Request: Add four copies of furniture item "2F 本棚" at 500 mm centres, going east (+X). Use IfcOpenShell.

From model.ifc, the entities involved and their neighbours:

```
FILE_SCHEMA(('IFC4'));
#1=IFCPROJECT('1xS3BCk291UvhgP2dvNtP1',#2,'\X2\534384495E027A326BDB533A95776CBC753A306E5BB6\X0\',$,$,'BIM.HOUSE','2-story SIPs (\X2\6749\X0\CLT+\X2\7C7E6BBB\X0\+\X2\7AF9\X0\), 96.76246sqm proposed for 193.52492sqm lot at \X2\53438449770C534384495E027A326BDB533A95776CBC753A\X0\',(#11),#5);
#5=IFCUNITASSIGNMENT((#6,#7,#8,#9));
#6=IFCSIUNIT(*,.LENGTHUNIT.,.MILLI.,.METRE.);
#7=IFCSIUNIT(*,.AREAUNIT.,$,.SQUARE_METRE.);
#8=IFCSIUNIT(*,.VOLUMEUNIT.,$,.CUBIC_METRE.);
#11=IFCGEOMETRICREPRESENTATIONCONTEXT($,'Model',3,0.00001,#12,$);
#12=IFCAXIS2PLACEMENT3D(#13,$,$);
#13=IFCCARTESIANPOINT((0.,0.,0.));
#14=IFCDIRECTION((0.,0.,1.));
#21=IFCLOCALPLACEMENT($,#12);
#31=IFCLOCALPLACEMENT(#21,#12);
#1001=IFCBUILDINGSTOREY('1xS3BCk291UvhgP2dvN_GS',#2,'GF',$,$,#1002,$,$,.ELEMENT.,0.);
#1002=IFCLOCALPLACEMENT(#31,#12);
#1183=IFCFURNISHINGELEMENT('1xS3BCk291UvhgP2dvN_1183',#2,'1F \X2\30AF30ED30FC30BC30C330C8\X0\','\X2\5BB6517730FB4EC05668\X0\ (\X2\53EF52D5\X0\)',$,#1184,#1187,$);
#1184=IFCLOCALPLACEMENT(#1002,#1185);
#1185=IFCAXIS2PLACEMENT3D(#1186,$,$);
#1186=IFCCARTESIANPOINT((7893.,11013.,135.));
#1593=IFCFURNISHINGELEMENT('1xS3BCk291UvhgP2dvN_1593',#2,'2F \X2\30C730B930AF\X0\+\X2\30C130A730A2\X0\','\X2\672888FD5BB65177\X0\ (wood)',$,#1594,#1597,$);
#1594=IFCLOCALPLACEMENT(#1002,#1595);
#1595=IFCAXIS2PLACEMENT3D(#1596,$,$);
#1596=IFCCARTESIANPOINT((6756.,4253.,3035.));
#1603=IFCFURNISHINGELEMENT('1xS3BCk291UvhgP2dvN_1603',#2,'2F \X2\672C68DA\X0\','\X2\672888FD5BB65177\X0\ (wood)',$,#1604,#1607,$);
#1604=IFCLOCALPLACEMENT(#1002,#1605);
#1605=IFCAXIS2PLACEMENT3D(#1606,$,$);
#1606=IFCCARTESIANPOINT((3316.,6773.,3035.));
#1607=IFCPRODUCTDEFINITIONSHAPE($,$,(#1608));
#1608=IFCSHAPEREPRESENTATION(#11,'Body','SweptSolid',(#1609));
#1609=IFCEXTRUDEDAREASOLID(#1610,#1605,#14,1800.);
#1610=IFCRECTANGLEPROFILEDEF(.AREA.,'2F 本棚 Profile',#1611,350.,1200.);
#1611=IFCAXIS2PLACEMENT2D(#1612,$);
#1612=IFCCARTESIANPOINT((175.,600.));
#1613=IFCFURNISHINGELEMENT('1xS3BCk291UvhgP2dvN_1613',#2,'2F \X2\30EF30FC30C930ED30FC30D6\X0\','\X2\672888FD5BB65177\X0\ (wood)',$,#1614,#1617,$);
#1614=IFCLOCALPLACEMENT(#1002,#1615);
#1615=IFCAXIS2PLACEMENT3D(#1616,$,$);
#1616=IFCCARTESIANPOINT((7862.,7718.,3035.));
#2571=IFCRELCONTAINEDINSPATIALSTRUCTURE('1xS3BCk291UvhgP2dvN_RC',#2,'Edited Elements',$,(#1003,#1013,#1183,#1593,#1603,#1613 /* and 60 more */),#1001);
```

```python
import numpy as np
import ifcopenshell
import ifcopenshell.api.geometry
import ifcopenshell.api.root
import ifcopenshell.util.element
import ifcopenshell.util.placement

model = ifcopenshell.open("model.ifc")


def reuse_history(source, copy):
    """copy_class also copies each property set's owner history, people and application; keep the originals."""
    for rel in copy.IsDefinedBy:
        if rel.is_a("IfcRelDefinesByProperties") and (history := rel.RelatingPropertyDefinition.OwnerHistory):
            rel.RelatingPropertyDefinition.OwnerHistory = source.OwnerHistory
            ifcopenshell.util.element.remove_deep2(model, history)


source = model.by_id(1603)
base = ifcopenshell.util.placement.get_local_placement(source.ObjectPlacement)
step = np.array([1.0, 0.0, 0.0]) * 500.0

for i in range(1, 5):
    copy = ifcopenshell.api.root.copy_class(model, product=source)
    copy.Representation = ifcopenshell.util.element.copy_deep(
        model, source.Representation, exclude=["IfcGeometricRepresentationContext", "IfcRepresentationMap"]
    )
    reuse_history(source, copy)
    matrix = base.copy()
    matrix[:3, 3] += i * step
    print("added at", matrix[:3, 3].round(3) + 0.0)
    ifcopenshell.api.geometry.edit_object_placement(model, product=copy, matrix=matrix, is_si=False)

model.write("model_rev.ifc")
```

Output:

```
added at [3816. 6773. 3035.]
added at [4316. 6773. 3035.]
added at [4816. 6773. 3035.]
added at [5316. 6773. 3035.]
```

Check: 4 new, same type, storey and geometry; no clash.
